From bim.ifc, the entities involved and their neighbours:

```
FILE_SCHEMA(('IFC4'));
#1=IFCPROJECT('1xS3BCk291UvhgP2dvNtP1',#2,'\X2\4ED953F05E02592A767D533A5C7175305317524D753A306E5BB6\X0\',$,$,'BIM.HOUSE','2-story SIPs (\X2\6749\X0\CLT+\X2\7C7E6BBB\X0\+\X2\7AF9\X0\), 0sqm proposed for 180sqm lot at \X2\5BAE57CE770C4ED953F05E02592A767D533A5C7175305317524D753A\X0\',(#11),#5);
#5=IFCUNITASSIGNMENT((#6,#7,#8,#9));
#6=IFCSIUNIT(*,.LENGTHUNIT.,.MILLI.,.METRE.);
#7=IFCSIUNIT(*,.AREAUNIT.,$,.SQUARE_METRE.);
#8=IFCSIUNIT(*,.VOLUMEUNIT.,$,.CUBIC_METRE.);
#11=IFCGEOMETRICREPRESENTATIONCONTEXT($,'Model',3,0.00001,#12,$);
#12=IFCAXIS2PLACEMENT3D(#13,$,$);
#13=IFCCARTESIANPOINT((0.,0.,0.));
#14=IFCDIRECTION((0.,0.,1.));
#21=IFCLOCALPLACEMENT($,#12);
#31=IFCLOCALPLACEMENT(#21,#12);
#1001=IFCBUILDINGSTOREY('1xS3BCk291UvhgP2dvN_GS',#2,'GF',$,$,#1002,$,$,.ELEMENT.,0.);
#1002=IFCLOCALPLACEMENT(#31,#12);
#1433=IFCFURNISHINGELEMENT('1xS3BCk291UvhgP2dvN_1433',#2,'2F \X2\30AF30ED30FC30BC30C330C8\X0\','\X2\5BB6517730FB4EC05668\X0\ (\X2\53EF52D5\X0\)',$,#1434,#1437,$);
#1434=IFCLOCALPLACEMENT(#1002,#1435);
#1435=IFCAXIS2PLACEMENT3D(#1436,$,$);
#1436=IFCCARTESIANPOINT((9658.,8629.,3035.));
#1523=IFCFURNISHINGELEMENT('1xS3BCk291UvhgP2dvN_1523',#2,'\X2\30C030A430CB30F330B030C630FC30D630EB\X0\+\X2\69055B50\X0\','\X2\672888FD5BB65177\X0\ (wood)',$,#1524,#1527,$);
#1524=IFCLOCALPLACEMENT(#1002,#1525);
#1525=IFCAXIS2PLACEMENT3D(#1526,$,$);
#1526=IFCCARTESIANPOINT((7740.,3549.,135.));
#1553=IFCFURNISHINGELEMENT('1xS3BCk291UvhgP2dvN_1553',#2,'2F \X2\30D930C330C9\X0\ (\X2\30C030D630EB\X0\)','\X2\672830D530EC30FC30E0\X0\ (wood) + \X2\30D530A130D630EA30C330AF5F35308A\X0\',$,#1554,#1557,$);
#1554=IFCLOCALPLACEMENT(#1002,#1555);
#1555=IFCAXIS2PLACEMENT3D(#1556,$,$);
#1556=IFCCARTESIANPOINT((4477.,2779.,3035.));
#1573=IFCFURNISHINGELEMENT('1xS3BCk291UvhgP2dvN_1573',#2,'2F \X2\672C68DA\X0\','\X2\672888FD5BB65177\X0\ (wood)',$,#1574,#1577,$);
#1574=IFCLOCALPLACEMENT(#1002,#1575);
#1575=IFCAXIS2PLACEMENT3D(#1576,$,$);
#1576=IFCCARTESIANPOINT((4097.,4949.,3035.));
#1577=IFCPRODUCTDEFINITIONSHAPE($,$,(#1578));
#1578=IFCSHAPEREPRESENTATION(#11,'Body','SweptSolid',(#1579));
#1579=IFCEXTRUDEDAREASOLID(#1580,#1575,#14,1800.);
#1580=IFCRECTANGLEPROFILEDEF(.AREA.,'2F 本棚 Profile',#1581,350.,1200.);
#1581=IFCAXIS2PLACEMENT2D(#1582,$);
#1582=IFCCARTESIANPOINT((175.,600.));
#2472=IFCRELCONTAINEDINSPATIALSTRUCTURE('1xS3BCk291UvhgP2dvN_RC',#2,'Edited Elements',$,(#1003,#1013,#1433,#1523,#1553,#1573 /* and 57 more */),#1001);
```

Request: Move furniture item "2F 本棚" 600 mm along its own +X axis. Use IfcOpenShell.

```python
import ifcopenshell
import ifcopenshell.api.geometry
import ifcopenshell.util.placement

model = ifcopenshell.open("bim.ifc")

item = model.by_id(1573)
matrix = ifcopenshell.util.placement.get_local_placement(item.ObjectPlacement)
matrix[:3, 3] += matrix[:3, 0] * 600.0
ifcopenshell.api.geometry.edit_object_placement(model, product=item, matrix=matrix, is_si=False)

print(ifcopenshell.util.placement.get_local_placement(item.ObjectPlacement).round(3) + 0.0)

model.write("bim_edited.ifc")
```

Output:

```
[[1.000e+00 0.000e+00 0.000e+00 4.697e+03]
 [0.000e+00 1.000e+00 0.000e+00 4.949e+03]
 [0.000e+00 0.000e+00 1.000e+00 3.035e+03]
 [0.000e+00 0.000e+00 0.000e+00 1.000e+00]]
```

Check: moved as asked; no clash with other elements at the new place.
